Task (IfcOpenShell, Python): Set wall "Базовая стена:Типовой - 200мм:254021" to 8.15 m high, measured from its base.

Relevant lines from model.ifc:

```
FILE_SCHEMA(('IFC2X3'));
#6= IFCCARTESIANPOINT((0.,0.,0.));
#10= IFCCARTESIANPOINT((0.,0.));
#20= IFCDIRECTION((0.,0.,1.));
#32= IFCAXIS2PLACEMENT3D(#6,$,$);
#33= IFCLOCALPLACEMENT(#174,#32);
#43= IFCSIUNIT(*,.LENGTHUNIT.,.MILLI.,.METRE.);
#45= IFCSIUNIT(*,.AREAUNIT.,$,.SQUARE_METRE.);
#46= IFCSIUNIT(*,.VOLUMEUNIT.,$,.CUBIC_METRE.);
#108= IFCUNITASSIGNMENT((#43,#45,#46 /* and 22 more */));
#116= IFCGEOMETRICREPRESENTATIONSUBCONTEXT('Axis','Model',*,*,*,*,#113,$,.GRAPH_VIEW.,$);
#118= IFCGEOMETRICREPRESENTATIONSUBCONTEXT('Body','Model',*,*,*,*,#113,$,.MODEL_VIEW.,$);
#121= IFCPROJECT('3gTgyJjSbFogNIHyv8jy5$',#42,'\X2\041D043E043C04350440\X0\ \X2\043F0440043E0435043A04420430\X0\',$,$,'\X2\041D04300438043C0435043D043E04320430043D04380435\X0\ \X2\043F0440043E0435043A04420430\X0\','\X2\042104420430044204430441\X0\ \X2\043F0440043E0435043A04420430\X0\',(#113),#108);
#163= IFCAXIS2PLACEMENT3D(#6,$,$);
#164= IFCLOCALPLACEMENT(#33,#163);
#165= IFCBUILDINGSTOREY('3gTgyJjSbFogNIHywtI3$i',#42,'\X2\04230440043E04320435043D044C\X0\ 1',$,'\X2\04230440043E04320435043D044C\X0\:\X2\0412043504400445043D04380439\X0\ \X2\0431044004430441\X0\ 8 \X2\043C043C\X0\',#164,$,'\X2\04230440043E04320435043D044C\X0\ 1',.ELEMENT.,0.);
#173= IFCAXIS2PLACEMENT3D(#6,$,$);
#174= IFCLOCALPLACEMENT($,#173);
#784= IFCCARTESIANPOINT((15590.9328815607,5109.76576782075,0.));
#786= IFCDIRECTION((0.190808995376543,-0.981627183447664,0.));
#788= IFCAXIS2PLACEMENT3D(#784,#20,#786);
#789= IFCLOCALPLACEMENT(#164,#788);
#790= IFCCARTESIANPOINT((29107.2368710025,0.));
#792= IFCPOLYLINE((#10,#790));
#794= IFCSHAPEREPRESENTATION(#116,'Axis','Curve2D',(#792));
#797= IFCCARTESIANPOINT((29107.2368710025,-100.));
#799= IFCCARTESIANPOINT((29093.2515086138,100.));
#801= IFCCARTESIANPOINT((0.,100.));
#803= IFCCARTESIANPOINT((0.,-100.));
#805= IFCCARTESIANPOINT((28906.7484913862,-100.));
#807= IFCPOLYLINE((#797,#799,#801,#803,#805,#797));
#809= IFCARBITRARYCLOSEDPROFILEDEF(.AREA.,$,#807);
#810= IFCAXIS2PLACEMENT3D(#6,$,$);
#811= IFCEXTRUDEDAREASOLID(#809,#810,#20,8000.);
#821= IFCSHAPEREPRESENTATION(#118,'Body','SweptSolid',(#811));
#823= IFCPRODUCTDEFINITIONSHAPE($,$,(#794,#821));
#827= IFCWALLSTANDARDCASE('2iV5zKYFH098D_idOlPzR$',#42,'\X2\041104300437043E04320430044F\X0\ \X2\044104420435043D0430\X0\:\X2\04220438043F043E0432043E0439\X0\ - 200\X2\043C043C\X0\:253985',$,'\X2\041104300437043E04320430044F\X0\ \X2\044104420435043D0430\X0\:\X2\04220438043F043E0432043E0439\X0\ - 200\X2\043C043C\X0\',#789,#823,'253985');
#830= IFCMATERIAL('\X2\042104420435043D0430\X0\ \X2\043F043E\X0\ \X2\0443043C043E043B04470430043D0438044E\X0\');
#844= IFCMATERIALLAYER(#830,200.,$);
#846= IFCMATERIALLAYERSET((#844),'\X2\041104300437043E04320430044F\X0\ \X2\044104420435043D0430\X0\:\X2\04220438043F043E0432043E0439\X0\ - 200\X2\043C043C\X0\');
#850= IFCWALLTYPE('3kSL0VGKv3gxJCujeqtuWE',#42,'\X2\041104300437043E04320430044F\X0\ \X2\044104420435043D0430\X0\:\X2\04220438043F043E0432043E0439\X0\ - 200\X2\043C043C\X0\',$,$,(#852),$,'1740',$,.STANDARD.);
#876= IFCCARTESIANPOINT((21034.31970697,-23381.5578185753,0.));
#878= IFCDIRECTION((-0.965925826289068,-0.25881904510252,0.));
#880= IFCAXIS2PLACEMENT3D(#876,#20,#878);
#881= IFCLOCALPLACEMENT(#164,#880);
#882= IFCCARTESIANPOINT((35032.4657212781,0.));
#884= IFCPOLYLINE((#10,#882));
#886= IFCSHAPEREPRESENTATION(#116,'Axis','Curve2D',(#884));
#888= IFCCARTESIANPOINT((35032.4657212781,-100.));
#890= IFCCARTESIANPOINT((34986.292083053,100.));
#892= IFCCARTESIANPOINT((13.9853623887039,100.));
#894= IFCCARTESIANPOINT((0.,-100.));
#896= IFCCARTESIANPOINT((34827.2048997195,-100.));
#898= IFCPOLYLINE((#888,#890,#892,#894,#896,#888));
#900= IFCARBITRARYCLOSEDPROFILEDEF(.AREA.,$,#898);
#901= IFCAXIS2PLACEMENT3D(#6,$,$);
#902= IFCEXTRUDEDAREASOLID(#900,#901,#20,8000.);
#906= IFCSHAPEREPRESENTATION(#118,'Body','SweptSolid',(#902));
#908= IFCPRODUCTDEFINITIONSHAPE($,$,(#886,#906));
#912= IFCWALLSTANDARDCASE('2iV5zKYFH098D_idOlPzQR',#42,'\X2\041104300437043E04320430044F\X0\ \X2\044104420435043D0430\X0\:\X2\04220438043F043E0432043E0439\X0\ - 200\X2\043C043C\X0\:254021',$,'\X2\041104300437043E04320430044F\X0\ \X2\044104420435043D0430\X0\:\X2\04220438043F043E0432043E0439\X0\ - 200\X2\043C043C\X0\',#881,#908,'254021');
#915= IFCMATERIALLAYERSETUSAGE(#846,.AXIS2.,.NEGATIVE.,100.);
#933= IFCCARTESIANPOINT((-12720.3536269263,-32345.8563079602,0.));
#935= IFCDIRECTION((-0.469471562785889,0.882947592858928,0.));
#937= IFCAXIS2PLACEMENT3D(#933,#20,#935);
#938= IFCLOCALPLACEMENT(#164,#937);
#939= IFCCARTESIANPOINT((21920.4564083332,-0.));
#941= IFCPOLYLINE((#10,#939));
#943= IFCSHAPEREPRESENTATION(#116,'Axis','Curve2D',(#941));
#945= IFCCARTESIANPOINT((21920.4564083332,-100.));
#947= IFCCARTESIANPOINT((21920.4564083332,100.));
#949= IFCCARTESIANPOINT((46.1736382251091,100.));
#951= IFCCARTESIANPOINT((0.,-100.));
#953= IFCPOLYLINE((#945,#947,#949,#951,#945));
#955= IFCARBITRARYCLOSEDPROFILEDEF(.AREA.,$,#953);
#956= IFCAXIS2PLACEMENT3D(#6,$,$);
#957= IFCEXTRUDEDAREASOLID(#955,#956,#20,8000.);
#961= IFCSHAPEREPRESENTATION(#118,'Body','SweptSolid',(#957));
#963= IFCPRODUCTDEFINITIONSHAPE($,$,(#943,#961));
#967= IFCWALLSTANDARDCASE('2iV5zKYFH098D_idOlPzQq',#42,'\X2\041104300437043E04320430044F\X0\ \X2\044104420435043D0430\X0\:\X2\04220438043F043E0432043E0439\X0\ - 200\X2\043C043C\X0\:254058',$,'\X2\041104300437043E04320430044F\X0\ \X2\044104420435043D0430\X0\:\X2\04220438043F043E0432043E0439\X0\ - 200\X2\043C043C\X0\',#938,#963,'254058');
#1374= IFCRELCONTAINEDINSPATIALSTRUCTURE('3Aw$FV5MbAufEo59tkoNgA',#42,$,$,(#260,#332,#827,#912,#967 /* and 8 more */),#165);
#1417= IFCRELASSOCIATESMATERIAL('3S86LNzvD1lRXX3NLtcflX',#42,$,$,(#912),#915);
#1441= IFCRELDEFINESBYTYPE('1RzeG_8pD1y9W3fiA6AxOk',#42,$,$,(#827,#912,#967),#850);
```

```python
import ifcopenshell
import ifcopenshell.geom
import ifcopenshell.util.representation
import ifcopenshell.util.shape
import ifcopenshell.util.unit

model = ifcopenshell.open("model.ifc")
unit_scale = ifcopenshell.util.unit.calculate_unit_scale(model)
settings = ifcopenshell.geom.settings()


def volume(element):
    """Net volume in cubic metres, openings subtracted."""
    shape = ifcopenshell.geom.create_shape(settings, element)
    return ifcopenshell.util.shape.get_volume(shape.geometry)


wall = model.by_id(912)
before = volume(wall)

body = ifcopenshell.util.representation.get_representation(wall, "Model", "Body")
solid = body.Items[0]
old_height = solid.Depth
solid.Depth = 8.15 / unit_scale
after = volume(wall)

print(f"height {old_height:g} -> {solid.Depth:g}, volume {before:.3f} -> {after:.3f} m3")

model.write("model_edited.ifc")
```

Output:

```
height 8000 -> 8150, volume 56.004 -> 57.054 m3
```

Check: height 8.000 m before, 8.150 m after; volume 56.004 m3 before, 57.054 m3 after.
